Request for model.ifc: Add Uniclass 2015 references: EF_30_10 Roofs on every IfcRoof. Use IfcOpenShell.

First a look at what the model holds.

```python
import ifcopenshell

model = ifcopenshell.open("model.ifc")
print(model.schema)
print("classifications:", [c.Name for c in model.by_type("IfcClassification")])
for ifc_class in ("IfcDoor", "IfcRoof", "IfcStair", "IfcWall", "IfcWindow"):
    print(ifc_class, len(model.by_type(ifc_class)))
```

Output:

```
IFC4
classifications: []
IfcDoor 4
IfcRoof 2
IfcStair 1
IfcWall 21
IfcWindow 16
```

```python
import ifcopenshell
import ifcopenshell.api.classification

model = ifcopenshell.open("model.ifc")

system = ifcopenshell.api.classification.add_classification(model, classification="Uniclass 2015")

codes = {
    "IfcRoof": ("EF_30_10", "Roofs"),
}
for ifc_class, (code, name) in codes.items():
    products = model.by_type(ifc_class)
    ifcopenshell.api.classification.add_reference(
        model, products=products, classification=system, identification=code, name=name
    )
    print(code, len(products))

model.write("model_updated.ifc")
```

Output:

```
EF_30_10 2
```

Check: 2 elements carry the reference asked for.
